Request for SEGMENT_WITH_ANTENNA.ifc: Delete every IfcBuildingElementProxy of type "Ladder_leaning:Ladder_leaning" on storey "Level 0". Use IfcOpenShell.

First a look at what the model holds.

```python
import ifcopenshell
import ifcopenshell.util.element

model = ifcopenshell.open("SEGMENT_WITH_ANTENNA.ifc")
print(model.schema)
storey = next(s for s in model.by_type("IfcBuildingStorey") if s.Name == "Level 0")
proxies = [e for e in ifcopenshell.util.element.get_decomposition(storey) if e.is_a("IfcBuildingElementProxy")]
seen = {}
for e in proxies:
    element_type = ifcopenshell.util.element.get_type(e)
    name = element_type.Name if element_type not in (None, e) else None
    seen[name] = seen.get(name, 0) + 1
for name, count in sorted(seen.items(), key=str):
    print(count, "x", name)
```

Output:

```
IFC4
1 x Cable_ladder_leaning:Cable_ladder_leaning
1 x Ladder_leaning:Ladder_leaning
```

```python
import ifcopenshell
import ifcopenshell.api.root
import ifcopenshell.util.element

model = ifcopenshell.open("SEGMENT_WITH_ANTENNA.ifc")

storey = next(s for s in model.by_type("IfcBuildingStorey") if s.Name == "Level 0")
proxies = [e for e in ifcopenshell.util.element.get_decomposition(storey) if e.is_a("IfcBuildingElementProxy")]
targets = [e for e in proxies if (t := ifcopenshell.util.element.get_type(e)) not in (None, e) and t.Name == "Ladder_leaning:Ladder_leaning"]

for e in targets:
    ifcopenshell.api.root.remove_product(model, product=e)
print(len(targets), "removed")

model.write("SEGMENT_WITH_ANTENNA-out.ifc")
```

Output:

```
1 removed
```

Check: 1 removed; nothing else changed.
